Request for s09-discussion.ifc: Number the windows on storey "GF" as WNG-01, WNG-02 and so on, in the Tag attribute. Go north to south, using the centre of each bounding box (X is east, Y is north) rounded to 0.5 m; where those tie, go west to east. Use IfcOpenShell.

First a look at what the model holds.

```python
import ifcopenshell
import ifcopenshell.util.element
import ifcopenshell.util.placement

model = ifcopenshell.open("s09-discussion.ifc")
print(model.schema)
storey = next(s for s in model.by_type("IfcBuildingStorey") if s.Name == "GF")
windows = [e for e in ifcopenshell.util.element.get_decomposition(storey) if e.is_a("IfcWindow")]
for e in sorted(windows, key=lambda e: e.id()):
    origin = ifcopenshell.util.placement.get_local_placement(e.ObjectPlacement)[:3, 3]
    print(e.id(), e.Tag, e.Name, origin.round(2) + 0.0, sep=" | ")
```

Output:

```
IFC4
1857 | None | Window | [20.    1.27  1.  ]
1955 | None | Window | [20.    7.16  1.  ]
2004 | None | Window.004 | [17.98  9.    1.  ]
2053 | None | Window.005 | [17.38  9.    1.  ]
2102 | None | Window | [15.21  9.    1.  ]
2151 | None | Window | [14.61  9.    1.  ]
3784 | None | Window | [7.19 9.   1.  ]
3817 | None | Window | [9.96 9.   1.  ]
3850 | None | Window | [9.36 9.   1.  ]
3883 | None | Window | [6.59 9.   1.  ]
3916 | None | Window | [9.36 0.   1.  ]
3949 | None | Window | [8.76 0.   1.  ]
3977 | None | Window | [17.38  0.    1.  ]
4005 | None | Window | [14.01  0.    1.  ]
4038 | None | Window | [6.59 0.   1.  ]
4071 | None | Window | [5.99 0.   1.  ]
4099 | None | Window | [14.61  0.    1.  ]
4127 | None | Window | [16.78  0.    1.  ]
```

```python
import ifcopenshell
import ifcopenshell.geom
import ifcopenshell.util.element
import ifcopenshell.util.shape

model = ifcopenshell.open("s09-discussion.ifc")
settings = ifcopenshell.geom.settings()
settings.set("use-world-coords", True)


def centre(element):
    shape = ifcopenshell.geom.create_shape(settings, element)
    return ifcopenshell.util.shape.get_bbox_centroid(shape.geometry)


storey = next(s for s in model.by_type("IfcBuildingStorey") if s.Name == "GF")
windows = [e for e in ifcopenshell.util.element.get_decomposition(storey) if e.is_a("IfcWindow")]

# Insertion points can sit at a corner or the storey origin, so sort by the geometry (in metres).
centres = {e: centre(e) for e in windows}
windows.sort(key=lambda e: (-round(centres[e][1] / 0.5), centres[e][0]))

for i, e in enumerate(windows, start=1):
    number = f"WNG-{i:02d}"
    e.Tag = number
    print(e.id(), number)

model.write("s09-discussion_updated.ifc")
```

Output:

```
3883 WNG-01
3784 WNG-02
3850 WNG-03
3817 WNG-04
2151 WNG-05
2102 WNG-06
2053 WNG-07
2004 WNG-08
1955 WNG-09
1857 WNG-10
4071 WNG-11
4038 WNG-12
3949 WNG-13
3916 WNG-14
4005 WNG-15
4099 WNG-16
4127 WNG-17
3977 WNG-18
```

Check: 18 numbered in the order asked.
